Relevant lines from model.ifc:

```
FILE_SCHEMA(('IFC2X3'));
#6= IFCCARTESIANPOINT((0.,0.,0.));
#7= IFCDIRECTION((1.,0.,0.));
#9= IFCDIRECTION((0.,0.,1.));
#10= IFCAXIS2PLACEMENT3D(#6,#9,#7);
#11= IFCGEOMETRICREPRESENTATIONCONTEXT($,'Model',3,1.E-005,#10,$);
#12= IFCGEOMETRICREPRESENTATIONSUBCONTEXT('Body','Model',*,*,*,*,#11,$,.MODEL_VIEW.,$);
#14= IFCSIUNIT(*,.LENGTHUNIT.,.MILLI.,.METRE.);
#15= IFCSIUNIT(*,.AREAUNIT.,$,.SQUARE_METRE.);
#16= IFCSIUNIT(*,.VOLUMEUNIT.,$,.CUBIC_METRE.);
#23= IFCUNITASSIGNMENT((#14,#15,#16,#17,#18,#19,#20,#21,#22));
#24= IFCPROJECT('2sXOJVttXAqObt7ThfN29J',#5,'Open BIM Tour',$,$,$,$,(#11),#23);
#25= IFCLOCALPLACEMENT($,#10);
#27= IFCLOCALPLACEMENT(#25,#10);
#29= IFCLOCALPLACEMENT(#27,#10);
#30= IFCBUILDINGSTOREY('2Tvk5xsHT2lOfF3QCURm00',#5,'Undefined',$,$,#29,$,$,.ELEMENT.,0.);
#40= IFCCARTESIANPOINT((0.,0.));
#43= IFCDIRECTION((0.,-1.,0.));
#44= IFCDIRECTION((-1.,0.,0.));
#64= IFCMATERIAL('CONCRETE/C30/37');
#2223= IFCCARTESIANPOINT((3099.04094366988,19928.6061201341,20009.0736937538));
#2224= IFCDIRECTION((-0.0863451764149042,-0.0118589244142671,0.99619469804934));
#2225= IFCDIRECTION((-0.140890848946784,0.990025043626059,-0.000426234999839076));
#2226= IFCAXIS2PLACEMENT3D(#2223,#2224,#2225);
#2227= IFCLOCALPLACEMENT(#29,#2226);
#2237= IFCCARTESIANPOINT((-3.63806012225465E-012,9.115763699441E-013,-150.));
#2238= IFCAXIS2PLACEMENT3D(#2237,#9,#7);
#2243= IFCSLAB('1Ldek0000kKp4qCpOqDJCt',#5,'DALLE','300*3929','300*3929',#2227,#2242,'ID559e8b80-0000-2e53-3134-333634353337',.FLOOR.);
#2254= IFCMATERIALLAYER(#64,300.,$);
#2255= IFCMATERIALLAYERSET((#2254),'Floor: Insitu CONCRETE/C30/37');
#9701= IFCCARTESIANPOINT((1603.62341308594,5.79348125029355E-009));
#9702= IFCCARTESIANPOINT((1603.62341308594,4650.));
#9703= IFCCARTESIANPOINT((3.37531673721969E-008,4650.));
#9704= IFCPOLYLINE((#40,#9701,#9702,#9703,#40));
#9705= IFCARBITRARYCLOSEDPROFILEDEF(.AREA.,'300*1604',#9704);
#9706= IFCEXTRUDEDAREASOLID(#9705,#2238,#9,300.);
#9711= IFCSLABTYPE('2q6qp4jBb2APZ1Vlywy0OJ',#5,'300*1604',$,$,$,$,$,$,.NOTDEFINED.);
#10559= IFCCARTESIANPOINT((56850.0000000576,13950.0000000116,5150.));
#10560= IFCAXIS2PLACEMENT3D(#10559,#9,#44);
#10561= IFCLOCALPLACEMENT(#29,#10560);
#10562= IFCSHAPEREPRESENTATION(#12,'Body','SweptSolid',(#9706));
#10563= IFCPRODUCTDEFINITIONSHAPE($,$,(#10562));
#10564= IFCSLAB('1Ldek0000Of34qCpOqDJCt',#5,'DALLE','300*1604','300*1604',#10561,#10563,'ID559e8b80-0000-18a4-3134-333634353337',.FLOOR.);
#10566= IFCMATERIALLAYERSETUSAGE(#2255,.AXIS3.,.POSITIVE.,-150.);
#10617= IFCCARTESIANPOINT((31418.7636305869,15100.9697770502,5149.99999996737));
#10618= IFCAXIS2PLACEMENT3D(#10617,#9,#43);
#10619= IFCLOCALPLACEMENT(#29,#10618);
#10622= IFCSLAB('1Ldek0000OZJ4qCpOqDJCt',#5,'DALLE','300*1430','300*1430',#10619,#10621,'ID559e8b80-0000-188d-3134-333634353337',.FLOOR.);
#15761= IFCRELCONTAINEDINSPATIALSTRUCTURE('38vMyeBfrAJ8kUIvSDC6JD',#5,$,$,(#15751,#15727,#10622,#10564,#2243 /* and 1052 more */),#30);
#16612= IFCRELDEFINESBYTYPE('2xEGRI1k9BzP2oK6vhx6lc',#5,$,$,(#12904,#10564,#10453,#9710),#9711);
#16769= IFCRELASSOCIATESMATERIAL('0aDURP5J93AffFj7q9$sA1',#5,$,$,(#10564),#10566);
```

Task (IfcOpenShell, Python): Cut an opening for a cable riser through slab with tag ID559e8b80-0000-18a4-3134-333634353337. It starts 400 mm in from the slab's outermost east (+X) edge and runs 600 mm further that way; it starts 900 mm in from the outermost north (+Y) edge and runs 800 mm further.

```python
import numpy as np
import ifcopenshell
import ifcopenshell.api.feature
import ifcopenshell.api.geometry
import ifcopenshell.api.root
import ifcopenshell.geom
import ifcopenshell.util.placement
import ifcopenshell.util.representation
import ifcopenshell.util.shape
import ifcopenshell.util.unit

model = ifcopenshell.open("model.ifc")
unit_scale = ifcopenshell.util.unit.calculate_unit_scale(model)
settings = ifcopenshell.geom.settings()


def volume(element):
    """Net volume in cubic metres, openings subtracted."""
    shape = ifcopenshell.geom.create_shape(settings, element)
    return ifcopenshell.util.shape.get_volume(shape.geometry)


slab = model.by_guid("1Ldek0000Of34qCpOqDJCt")
before = volume(slab)

# Extent in the slab's own axes, in metres. The edges named are its -X and -Y sides.
slab_shape = ifcopenshell.geom.create_shape(settings, slab)
vertices = ifcopenshell.util.shape.get_vertices(slab_shape.geometry)
x_min, y_min, bottom = vertices.min(axis=0)
top = vertices[:, 2].max()

opening = ifcopenshell.api.root.create_entity(model, ifc_class="IfcOpeningElement", name="Cable riser opening")
context = ifcopenshell.util.representation.get_context(model, "Model", "Body", "MODEL_VIEW")
width, depth = 0.6, 0.8
outline = [(0.0, 0.0), (width, 0.0), (width, depth), (0.0, depth), (0.0, 0.0)]
# Overshoot both faces by 50 mm so the cut is clean.
shape = ifcopenshell.api.geometry.add_slab_representation(
    model, context=context, depth=top - bottom + 0.1, polyline=outline
)
ifcopenshell.api.geometry.assign_representation(model, product=opening, representation=shape)

matrix = ifcopenshell.util.placement.get_local_placement(slab.ObjectPlacement)
matrix[:, 3] = matrix @ np.append(np.array([x_min + 0.4, y_min + 0.9, bottom - 0.05]) / unit_scale, 1.0)
ifcopenshell.api.geometry.edit_object_placement(model, product=opening, matrix=matrix, is_si=False)
ifcopenshell.api.feature.add_feature(model, feature=opening, element=slab)

after = volume(slab)

print(f"slab volume {before:.3f} -> {after:.3f} m3")

model.write("model-out.ifc")
```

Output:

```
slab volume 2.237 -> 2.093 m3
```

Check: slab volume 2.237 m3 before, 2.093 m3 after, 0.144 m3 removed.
